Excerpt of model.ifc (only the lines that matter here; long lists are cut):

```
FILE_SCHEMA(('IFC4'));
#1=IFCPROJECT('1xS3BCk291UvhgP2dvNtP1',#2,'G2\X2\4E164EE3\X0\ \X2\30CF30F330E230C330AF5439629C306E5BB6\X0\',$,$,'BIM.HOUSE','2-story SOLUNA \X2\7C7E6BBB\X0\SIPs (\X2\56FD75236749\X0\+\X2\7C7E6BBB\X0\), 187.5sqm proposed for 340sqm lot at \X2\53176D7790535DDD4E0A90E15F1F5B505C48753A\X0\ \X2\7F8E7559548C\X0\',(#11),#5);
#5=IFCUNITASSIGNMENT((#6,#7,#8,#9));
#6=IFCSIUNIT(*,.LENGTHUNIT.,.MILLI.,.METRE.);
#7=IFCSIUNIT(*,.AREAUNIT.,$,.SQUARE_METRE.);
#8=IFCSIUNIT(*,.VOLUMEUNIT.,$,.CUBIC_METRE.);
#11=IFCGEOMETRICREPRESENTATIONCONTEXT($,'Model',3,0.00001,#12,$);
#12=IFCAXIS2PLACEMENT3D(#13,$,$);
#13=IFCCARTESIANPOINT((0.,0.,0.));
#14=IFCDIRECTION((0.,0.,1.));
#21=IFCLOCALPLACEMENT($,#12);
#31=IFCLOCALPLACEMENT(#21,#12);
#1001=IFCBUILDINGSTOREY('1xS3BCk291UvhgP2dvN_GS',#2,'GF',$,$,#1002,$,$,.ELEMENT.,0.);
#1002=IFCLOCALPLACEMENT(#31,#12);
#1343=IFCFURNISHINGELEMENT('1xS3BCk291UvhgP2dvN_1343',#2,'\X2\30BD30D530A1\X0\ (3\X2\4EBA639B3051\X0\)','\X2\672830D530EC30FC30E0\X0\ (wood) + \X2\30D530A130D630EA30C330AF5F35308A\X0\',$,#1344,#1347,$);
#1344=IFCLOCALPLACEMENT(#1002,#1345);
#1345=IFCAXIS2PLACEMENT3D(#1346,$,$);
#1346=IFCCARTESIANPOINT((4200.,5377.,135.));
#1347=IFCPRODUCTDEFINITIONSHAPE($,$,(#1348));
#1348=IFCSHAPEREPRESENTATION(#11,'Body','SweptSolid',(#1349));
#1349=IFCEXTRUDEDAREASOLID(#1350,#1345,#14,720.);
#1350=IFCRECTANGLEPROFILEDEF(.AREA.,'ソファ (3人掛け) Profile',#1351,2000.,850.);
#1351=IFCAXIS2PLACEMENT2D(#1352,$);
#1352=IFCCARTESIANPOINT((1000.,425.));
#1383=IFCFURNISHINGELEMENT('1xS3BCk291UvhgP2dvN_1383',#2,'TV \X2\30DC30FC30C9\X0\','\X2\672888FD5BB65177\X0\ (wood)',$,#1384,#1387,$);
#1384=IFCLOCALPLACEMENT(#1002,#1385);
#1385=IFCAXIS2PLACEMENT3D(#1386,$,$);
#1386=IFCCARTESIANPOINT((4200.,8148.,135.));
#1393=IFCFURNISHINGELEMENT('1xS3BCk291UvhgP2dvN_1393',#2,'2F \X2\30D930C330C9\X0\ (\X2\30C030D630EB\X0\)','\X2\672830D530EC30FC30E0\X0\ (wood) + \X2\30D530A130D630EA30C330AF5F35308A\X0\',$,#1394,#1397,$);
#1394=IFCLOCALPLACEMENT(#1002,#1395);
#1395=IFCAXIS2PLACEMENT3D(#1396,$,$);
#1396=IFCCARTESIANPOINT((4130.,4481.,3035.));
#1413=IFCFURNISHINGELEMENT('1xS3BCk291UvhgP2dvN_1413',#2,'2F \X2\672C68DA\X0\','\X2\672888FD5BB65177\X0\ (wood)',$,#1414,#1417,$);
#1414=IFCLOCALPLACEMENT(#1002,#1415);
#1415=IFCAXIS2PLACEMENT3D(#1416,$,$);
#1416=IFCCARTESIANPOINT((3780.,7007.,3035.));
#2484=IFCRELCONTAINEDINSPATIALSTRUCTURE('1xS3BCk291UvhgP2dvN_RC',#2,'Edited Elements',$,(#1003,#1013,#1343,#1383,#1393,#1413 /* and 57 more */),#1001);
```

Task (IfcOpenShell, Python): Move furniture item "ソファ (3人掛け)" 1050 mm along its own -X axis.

```python
import ifcopenshell
import ifcopenshell.api.geometry
import ifcopenshell.util.placement

model = ifcopenshell.open("model.ifc")

item = model.by_id(1343)
matrix = ifcopenshell.util.placement.get_local_placement(item.ObjectPlacement)
matrix[:3, 3] -= matrix[:3, 0] * 1050.0
ifcopenshell.api.geometry.edit_object_placement(model, product=item, matrix=matrix, is_si=False)

print(ifcopenshell.util.placement.get_local_placement(item.ObjectPlacement).round(3) + 0.0)

model.write("model_edited.ifc")
```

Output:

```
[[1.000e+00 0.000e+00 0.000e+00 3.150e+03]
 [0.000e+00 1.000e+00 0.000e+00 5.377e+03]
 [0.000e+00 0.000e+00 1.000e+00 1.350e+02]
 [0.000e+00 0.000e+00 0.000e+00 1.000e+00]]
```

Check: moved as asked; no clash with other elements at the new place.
